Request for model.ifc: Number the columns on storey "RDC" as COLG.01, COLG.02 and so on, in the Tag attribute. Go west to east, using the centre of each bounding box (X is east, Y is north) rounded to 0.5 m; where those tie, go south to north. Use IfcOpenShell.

First a look at what the model holds.

```python
import ifcopenshell
import ifcopenshell.util.element
import ifcopenshell.util.placement

model = ifcopenshell.open("model.ifc")
print(model.schema)
storey = next(s for s in model.by_type("IfcBuildingStorey") if s.Name == "RDC")
columns = [e for e in ifcopenshell.util.element.get_decomposition(storey) if e.is_a("IfcColumn")]
for e in sorted(columns, key=lambda e: e.id()):
    origin = ifcopenshell.util.placement.get_local_placement(e.ObjectPlacement)[:3, 3]
    print(e.id(), e.Tag, e.Name, origin.round(2) + 0.0, sep=" | ")
```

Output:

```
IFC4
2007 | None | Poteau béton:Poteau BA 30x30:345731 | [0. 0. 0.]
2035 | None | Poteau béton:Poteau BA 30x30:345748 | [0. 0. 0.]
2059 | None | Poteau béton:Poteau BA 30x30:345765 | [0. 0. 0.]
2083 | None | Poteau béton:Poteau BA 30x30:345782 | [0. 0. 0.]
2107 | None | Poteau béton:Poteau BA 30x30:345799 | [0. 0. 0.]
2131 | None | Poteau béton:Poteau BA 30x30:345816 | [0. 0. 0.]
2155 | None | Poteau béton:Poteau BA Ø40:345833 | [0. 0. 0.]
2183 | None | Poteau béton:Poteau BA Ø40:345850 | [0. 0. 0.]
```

```python
import ifcopenshell
import ifcopenshell.geom
import ifcopenshell.util.element
import ifcopenshell.util.shape

model = ifcopenshell.open("model.ifc")
settings = ifcopenshell.geom.settings()
settings.set("use-world-coords", True)


def centre(element):
    shape = ifcopenshell.geom.create_shape(settings, element)
    return ifcopenshell.util.shape.get_bbox_centroid(shape.geometry)


storey = next(s for s in model.by_type("IfcBuildingStorey") if s.Name == "RDC")
columns = [e for e in ifcopenshell.util.element.get_decomposition(storey) if e.is_a("IfcColumn")]

# Insertion points can sit at a corner or the storey origin, so sort by the geometry (in metres).
centres = {e: centre(e) for e in columns}
columns.sort(key=lambda e: (round(centres[e][0] / 0.5), centres[e][1]))

for i, e in enumerate(columns, start=1):
    number = f"COLG.{i:02d}"
    e.Tag = number
    print(e.id(), number)

model.write("model-out.ifc")
```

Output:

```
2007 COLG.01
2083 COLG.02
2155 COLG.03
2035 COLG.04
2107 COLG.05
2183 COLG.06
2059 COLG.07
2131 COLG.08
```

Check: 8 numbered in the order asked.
